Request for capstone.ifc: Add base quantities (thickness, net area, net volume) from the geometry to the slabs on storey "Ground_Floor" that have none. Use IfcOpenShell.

First a look at what the model holds.

```python
import ifcopenshell
import ifcopenshell.util.element
import ifcopenshell.util.unit

model = ifcopenshell.open("capstone.ifc")
print(model.schema)
for unit_type in ("LENGTHUNIT", "AREAUNIT", "VOLUMEUNIT"):
    print(unit_type, ifcopenshell.util.unit.calculate_unit_scale(model, unit_type))
storey = next(s for s in model.by_type("IfcBuildingStorey") if s.Name == "Ground_Floor")
slabs = [e for e in ifcopenshell.util.element.get_decomposition(storey) if e.is_a("IfcSlab")]
for e in sorted(slabs, key=lambda e: e.id()):
    print(e.id(), e.is_a(), e.Name, list(ifcopenshell.util.element.get_psets(e, qtos_only=True)), sep=" | ")
```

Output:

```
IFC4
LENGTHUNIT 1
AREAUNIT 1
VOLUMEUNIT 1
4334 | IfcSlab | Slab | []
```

```python
import ifcopenshell
import ifcopenshell.api.pset
import ifcopenshell.geom
import ifcopenshell.util.element
import ifcopenshell.util.shape
import ifcopenshell.util.unit

model = ifcopenshell.open("capstone.ifc")
unit_scale = ifcopenshell.util.unit.calculate_unit_scale(model)
area_scale = ifcopenshell.util.unit.calculate_unit_scale(model, "AREAUNIT")
volume_scale = ifcopenshell.util.unit.calculate_unit_scale(model, "VOLUMEUNIT")
settings = ifcopenshell.geom.settings()

storey = next(s for s in model.by_type("IfcBuildingStorey") if s.Name == "Ground_Floor")
slabs = [e for e in ifcopenshell.util.element.get_decomposition(storey) if e.is_a("IfcSlab")]

for e in sorted(slabs, key=lambda e: e.id()):
    if ifcopenshell.util.element.get_psets(e, qtos_only=True, should_inherit=False):
        continue
    # Geometry comes back in metres, in the element's own axes.
    shape = ifcopenshell.geom.create_shape(settings, e)
    values = {
        "Width": ifcopenshell.util.shape.get_z(shape.geometry) / unit_scale,
        "NetArea": ifcopenshell.util.shape.get_footprint_area(shape.geometry) / area_scale,
        "NetVolume": ifcopenshell.util.shape.get_volume(shape.geometry) / volume_scale,
    }
    qto = ifcopenshell.api.pset.add_qto(model, product=e, name="Qto_SlabBaseQuantities")
    ifcopenshell.api.pset.edit_qto(model, qto=qto, properties=values)
    print(e.id(), {k: round(v, 3) for k, v in values.items()})

model.write("capstone_edited.ifc")
```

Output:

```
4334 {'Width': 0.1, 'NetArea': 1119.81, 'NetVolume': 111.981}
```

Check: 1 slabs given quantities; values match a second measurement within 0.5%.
